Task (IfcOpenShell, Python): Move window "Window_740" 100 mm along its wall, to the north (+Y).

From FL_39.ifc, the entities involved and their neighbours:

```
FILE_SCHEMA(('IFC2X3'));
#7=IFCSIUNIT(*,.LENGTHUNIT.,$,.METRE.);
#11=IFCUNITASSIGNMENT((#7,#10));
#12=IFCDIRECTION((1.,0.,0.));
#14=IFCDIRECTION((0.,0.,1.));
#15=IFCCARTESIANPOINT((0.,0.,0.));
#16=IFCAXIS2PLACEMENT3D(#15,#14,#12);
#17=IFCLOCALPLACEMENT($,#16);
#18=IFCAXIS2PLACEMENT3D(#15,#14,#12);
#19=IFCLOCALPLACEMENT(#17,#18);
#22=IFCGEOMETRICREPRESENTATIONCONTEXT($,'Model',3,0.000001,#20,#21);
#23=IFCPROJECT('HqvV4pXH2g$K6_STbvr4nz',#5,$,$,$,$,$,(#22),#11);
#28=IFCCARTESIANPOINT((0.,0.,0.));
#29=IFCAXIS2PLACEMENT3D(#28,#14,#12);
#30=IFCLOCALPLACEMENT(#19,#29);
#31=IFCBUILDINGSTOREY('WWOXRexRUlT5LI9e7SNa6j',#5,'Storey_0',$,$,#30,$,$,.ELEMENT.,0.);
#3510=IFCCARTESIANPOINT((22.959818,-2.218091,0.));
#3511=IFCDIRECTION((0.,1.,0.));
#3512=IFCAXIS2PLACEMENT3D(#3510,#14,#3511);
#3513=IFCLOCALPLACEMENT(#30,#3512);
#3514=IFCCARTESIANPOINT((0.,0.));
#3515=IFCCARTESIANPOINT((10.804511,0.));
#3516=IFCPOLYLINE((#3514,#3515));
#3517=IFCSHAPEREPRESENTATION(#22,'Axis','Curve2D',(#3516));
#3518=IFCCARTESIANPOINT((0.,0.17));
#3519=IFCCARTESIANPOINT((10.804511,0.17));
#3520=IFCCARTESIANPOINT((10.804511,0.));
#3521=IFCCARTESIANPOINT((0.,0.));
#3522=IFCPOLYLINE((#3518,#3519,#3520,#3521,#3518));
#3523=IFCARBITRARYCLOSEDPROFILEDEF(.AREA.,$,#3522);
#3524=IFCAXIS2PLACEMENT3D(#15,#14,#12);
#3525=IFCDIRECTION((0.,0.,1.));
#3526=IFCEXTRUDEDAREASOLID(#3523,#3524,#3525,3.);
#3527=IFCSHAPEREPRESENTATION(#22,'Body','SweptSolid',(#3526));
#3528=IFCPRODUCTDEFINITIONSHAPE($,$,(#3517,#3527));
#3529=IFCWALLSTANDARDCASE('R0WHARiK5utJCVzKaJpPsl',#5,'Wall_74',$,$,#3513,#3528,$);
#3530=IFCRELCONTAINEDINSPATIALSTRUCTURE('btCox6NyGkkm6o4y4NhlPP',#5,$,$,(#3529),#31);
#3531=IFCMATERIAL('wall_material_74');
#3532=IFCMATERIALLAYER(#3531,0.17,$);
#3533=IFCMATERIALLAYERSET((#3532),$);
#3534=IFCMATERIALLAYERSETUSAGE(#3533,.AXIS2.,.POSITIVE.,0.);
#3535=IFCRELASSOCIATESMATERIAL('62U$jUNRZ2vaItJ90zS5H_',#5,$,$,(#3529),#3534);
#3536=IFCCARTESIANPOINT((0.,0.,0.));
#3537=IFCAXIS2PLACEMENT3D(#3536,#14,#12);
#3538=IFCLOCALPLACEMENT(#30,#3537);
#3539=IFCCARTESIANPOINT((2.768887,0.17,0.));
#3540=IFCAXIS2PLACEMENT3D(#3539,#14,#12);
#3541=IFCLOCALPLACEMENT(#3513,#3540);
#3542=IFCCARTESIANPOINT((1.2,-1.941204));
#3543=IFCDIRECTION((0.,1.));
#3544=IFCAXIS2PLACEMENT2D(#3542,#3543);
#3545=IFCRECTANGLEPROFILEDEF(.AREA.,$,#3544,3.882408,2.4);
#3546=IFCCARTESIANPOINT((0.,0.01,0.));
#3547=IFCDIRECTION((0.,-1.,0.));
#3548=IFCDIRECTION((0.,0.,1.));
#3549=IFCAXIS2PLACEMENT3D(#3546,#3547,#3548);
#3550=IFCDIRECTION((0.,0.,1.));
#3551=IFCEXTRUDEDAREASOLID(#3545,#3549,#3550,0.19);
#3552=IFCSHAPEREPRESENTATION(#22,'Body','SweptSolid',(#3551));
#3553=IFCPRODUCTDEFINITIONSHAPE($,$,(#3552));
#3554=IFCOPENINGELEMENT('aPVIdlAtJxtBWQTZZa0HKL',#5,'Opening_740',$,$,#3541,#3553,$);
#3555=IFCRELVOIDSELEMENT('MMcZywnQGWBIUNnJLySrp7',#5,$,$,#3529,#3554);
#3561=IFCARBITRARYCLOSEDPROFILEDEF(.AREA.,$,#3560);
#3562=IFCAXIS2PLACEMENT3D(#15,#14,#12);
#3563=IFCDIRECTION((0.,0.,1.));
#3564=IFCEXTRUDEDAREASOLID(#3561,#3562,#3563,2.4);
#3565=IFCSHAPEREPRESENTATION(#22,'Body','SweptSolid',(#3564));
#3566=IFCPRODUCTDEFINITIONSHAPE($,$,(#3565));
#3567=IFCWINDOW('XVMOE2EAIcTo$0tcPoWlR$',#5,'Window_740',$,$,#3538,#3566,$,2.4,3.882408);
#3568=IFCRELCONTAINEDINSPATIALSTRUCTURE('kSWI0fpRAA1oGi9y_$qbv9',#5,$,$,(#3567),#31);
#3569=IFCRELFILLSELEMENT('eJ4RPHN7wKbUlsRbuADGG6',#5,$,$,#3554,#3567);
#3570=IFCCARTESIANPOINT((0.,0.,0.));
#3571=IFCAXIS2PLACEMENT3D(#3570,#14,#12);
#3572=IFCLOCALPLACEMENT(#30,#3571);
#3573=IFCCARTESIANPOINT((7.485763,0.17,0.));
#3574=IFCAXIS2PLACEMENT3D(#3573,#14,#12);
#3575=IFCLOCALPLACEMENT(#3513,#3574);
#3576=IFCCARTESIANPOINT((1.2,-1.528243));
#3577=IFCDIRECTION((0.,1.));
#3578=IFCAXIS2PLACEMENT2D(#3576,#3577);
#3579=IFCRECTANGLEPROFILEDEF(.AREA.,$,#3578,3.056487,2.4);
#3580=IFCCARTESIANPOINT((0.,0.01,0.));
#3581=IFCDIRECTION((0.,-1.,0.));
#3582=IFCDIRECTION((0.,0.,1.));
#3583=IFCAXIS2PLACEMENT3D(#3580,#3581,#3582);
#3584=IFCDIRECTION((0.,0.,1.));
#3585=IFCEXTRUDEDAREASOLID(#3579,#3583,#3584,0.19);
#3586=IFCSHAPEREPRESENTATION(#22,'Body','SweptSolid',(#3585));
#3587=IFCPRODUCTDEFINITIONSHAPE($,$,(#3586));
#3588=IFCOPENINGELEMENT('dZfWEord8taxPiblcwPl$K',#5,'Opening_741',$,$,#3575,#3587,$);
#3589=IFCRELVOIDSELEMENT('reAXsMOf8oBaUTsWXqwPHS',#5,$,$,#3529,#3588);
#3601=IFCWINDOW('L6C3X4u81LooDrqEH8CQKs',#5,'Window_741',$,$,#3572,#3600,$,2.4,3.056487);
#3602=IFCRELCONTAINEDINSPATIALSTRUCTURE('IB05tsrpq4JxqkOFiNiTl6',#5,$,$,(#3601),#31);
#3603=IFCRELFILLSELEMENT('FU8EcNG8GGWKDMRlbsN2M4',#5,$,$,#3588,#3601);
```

```python
import ifcopenshell
import ifcopenshell.api.geometry
import ifcopenshell.util.placement
import ifcopenshell.util.unit

model = ifcopenshell.open("FL_39.ifc")
unit_scale = ifcopenshell.util.unit.calculate_unit_scale(model)

window = model.by_guid("XVMOE2EAIcTo$0tcPoWlR$")
opening = window.FillsVoids[0].RelatingOpeningElement
wall = opening.VoidsElements[0].RelatingBuildingElement

wall_matrix = ifcopenshell.util.placement.get_local_placement(wall.ObjectPlacement)
shift = wall_matrix[:3, 0] * 0.1 / unit_scale
before = ifcopenshell.util.placement.get_local_placement(window.ObjectPlacement)[:3, 3].copy()

# The window is not placed relative to its opening, so move both.
for product in (opening, window):
    matrix = ifcopenshell.util.placement.get_local_placement(product.ObjectPlacement)
    matrix[:3, 3] += shift
    ifcopenshell.api.geometry.edit_object_placement(model, product=product, matrix=matrix, is_si=False)

after = ifcopenshell.util.placement.get_local_placement(window.ObjectPlacement)[:3, 3]
print("window moved by", (after - before).round(3) + 0.0)

model.write("FL_39_updated.ifc")
```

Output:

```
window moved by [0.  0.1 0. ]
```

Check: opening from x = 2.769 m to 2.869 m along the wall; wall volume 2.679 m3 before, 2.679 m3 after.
